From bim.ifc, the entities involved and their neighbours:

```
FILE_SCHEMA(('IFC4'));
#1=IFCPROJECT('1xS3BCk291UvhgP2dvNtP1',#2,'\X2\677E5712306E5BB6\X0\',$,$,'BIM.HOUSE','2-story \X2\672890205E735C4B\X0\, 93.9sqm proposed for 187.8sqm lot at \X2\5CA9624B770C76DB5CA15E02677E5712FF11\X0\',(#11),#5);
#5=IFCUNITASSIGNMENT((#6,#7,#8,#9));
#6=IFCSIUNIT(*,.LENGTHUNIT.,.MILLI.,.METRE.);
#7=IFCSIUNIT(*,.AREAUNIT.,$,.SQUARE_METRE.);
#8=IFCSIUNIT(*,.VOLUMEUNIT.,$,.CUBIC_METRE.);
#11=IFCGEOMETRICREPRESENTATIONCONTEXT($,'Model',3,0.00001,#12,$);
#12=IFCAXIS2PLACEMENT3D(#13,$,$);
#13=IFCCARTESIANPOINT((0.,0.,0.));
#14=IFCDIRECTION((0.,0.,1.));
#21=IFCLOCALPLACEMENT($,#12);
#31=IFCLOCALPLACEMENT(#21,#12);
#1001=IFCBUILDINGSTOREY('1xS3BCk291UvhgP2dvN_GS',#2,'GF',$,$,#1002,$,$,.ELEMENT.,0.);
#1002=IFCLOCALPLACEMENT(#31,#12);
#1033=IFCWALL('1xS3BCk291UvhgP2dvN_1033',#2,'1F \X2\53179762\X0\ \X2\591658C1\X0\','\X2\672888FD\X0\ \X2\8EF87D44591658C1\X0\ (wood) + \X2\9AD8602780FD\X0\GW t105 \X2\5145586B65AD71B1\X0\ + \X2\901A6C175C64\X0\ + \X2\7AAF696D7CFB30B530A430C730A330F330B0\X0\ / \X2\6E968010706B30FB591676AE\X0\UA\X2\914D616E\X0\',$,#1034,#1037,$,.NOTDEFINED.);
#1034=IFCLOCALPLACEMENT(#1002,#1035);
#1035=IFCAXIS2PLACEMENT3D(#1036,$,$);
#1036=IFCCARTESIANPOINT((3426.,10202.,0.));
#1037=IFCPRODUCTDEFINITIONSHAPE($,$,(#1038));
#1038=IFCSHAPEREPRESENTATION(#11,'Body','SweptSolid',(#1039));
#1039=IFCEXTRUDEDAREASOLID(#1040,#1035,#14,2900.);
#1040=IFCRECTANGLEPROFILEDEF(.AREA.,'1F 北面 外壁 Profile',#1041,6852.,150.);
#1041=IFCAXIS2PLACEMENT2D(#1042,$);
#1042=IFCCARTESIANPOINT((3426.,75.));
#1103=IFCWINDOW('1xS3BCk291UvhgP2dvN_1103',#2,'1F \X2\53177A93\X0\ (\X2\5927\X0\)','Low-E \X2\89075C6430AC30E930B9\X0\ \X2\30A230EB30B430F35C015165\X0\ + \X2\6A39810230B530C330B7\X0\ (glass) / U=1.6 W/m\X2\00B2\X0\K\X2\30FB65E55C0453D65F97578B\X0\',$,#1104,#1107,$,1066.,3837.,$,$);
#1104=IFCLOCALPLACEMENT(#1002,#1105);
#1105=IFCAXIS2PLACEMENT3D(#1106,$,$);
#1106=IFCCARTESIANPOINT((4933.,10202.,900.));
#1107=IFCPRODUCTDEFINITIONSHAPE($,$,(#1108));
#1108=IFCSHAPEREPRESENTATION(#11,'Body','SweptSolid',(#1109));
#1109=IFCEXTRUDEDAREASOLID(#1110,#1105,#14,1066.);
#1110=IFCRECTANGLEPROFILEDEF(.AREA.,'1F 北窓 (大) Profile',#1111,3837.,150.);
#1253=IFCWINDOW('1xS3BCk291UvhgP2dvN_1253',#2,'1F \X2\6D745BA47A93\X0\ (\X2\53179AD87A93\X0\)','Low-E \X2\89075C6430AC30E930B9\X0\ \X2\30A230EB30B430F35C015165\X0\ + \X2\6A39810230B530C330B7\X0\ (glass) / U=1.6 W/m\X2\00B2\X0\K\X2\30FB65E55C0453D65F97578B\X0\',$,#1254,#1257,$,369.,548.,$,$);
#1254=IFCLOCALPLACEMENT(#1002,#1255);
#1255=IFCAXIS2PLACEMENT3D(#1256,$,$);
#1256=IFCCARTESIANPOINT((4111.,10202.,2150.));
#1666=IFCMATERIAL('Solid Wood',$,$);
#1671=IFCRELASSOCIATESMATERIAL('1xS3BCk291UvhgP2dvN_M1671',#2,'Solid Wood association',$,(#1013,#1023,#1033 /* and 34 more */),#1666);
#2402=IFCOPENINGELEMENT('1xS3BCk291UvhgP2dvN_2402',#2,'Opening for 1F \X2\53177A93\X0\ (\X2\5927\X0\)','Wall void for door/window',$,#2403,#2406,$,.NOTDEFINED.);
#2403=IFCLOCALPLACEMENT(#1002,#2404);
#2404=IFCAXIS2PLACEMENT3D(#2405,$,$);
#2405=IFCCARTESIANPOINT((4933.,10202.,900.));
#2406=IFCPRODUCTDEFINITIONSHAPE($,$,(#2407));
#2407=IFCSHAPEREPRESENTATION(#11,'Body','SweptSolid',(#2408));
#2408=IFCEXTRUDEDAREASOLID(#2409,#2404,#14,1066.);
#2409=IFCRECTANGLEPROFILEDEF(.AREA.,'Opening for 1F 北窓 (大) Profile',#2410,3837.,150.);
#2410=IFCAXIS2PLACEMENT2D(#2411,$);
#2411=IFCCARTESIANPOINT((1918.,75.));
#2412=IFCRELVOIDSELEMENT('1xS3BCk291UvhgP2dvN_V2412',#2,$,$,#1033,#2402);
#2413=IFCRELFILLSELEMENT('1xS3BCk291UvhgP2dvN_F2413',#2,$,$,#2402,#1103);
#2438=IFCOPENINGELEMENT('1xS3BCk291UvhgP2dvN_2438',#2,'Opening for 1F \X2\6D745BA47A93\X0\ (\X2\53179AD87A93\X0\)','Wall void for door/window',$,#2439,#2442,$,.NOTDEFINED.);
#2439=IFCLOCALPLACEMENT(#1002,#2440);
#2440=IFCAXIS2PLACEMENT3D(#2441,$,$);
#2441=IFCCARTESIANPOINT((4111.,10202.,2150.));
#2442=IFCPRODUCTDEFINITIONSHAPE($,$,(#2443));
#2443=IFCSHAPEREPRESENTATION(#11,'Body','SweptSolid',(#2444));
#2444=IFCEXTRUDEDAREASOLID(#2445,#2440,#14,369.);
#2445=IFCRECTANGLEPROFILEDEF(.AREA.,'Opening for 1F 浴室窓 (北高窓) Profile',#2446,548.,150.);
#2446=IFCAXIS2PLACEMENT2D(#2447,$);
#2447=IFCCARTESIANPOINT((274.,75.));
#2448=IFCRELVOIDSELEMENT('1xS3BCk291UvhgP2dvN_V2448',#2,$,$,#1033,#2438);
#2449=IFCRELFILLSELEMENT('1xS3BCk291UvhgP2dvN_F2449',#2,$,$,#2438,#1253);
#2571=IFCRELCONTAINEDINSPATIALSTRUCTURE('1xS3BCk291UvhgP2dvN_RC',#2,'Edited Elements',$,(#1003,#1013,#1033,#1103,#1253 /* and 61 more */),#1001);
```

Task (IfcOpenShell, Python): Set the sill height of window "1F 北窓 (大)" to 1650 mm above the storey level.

```python
import numpy as np
import ifcopenshell
import ifcopenshell.api.geometry
import ifcopenshell.geom
import ifcopenshell.util.element
import ifcopenshell.util.placement
import ifcopenshell.util.shape
import ifcopenshell.util.unit

model = ifcopenshell.open("bim.ifc")
unit_scale = ifcopenshell.util.unit.calculate_unit_scale(model)

window = model.by_id(1103)
opening = window.FillsVoids[0].RelatingOpeningElement
storey = ifcopenshell.util.element.get_container(window, ifc_class="IfcBuildingStorey")
level = ifcopenshell.util.placement.get_local_placement(storey.ObjectPlacement)[2, 3]

# The opening's origin need not be at the sill, so measure its lowest point.
shape = ifcopenshell.geom.create_shape(ifcopenshell.geom.settings(), opening)
bottom = ifcopenshell.util.shape.get_shape_bottom_elevation(shape, shape.geometry) / unit_scale
dz = level + 1650.0 - bottom

shift = np.array([0.0, 0.0, dz])
# The window is not placed relative to its opening, so move both.
for product in (opening, window):
    matrix = ifcopenshell.util.placement.get_local_placement(product.ObjectPlacement)
    matrix[:3, 3] += shift
    ifcopenshell.api.geometry.edit_object_placement(model, product=product, matrix=matrix, is_si=False)

print(f"moved by {dz * unit_scale:+.3f} m")

model.write("bim_edited.ifc")
```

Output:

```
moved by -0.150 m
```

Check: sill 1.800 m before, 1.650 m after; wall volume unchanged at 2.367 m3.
